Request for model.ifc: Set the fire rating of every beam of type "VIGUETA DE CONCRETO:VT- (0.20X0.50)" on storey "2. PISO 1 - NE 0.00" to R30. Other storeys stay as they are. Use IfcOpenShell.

First a look at what the model holds.

```python
import ifcopenshell
import ifcopenshell.util.element

model = ifcopenshell.open("model.ifc")
print(model.schema)
storey = next(s for s in model.by_type("IfcBuildingStorey") if s.Name == "2. PISO 1 - NE 0.00")
beams = [e for e in ifcopenshell.util.element.get_decomposition(storey) if e.is_a("IfcBeam")]
seen = {}
for e in beams:
    element_type = ifcopenshell.util.element.get_type(e)
    key = (element_type.Name if element_type != e and element_type else None, ifcopenshell.util.element.get_pset(e, "Pset_BeamCommon", "FireRating"))
    seen[key] = seen.get(key, 0) + 1
for (name, value), count in sorted(seen.items(), key=str):
    print(count, "x", name, "|", value)
```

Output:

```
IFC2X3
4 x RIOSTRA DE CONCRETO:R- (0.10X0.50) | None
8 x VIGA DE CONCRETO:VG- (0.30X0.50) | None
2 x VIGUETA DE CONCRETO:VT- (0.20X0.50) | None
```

```python
import ifcopenshell
import ifcopenshell.api.pset
import ifcopenshell.util.element

model = ifcopenshell.open("model.ifc")

storey = next(s for s in model.by_type("IfcBuildingStorey") if s.Name == "2. PISO 1 - NE 0.00")
beams = [e for e in ifcopenshell.util.element.get_decomposition(storey) if e.is_a("IfcBeam")]

count = 0
for e in beams:
    element_type = ifcopenshell.util.element.get_type(e)
    if element_type in (None, e) or element_type.Name != "VIGUETA DE CONCRETO:VT- (0.20X0.50)":
        continue
    # add_pset returns the element's existing set when there is one.
    pset = ifcopenshell.api.pset.add_pset(model, product=e, name="Pset_BeamCommon")
    ifcopenshell.api.pset.edit_pset(model, pset=pset, properties={"FireRating": "R30"})
    count += 1

print(count, "beams updated")

model.write("model-out.ifc")
```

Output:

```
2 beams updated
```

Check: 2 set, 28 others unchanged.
